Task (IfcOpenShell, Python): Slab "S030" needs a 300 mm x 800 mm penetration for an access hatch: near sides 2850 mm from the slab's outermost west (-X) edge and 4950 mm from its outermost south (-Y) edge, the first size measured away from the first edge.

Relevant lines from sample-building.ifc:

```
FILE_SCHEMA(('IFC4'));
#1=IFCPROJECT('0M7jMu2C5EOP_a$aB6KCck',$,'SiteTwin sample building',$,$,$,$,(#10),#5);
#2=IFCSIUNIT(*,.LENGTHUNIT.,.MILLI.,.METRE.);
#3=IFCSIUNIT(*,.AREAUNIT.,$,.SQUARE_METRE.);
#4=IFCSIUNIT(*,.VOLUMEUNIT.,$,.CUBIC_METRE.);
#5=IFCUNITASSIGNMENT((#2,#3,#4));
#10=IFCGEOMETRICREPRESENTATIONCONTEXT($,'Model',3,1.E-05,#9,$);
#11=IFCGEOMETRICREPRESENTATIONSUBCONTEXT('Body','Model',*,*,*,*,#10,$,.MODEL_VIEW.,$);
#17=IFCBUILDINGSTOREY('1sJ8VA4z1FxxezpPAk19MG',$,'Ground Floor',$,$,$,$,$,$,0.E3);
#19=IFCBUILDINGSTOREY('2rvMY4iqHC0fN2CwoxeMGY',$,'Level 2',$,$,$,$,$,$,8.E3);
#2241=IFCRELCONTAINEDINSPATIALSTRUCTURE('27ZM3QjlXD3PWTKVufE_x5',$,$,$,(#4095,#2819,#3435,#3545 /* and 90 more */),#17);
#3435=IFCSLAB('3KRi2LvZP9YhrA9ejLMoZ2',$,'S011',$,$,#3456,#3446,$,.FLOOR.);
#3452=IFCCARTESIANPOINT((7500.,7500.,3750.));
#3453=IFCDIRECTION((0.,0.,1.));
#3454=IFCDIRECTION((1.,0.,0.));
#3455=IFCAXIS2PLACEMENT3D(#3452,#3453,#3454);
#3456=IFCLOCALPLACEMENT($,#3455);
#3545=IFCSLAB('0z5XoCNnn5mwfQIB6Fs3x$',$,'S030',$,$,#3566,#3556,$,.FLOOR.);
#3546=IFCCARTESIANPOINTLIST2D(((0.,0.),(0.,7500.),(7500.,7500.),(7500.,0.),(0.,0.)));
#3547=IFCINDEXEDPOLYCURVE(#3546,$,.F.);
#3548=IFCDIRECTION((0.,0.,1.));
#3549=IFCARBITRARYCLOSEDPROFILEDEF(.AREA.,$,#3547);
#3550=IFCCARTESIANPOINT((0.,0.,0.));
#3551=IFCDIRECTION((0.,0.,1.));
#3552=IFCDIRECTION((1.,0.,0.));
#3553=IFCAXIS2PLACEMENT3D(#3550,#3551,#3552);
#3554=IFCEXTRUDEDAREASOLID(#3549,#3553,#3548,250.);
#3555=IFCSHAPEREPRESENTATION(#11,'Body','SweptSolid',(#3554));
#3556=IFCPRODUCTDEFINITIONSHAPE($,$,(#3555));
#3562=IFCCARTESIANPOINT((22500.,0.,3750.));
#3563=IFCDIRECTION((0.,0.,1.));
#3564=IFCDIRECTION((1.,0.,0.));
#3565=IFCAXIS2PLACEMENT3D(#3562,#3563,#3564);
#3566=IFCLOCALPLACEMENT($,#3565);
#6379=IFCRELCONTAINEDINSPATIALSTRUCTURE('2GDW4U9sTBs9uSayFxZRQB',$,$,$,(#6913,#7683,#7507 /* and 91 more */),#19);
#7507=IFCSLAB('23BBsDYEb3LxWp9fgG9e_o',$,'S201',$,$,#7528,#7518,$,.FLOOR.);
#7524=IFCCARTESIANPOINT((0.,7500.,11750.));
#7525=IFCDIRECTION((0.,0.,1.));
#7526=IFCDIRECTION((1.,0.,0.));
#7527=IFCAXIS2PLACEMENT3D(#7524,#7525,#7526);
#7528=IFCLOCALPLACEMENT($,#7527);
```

```python
import numpy as np
import ifcopenshell
import ifcopenshell.api.feature
import ifcopenshell.api.geometry
import ifcopenshell.api.root
import ifcopenshell.geom
import ifcopenshell.util.placement
import ifcopenshell.util.representation
import ifcopenshell.util.shape
import ifcopenshell.util.unit

model = ifcopenshell.open("sample-building.ifc")
unit_scale = ifcopenshell.util.unit.calculate_unit_scale(model)
settings = ifcopenshell.geom.settings()


def volume(element):
    """Net volume in cubic metres, openings subtracted."""
    shape = ifcopenshell.geom.create_shape(settings, element)
    return ifcopenshell.util.shape.get_volume(shape.geometry)


slab = model.by_guid("0z5XoCNnn5mwfQIB6Fs3x$")
before = volume(slab)

# Extent in the slab's own axes, in metres. The edges named are its -X and -Y sides.
slab_shape = ifcopenshell.geom.create_shape(settings, slab)
vertices = ifcopenshell.util.shape.get_vertices(slab_shape.geometry)
x_min, y_min, bottom = vertices.min(axis=0)
top = vertices[:, 2].max()

opening = ifcopenshell.api.root.create_entity(model, ifc_class="IfcOpeningElement", name="Access hatch opening", predefined_type="OPENING")
context = ifcopenshell.util.representation.get_context(model, "Model", "Body", "MODEL_VIEW")
width, depth = 0.3, 0.8
outline = [(0.0, 0.0), (width, 0.0), (width, depth), (0.0, depth), (0.0, 0.0)]
# Overshoot both faces by 50 mm so the cut is clean.
shape = ifcopenshell.api.geometry.add_slab_representation(
    model, context=context, depth=top - bottom + 0.1, polyline=outline
)
ifcopenshell.api.geometry.assign_representation(model, product=opening, representation=shape)

matrix = ifcopenshell.util.placement.get_local_placement(slab.ObjectPlacement)
matrix[:, 3] = matrix @ np.append(np.array([x_min + 2.85, y_min + 4.95, bottom - 0.05]) / unit_scale, 1.0)
ifcopenshell.api.geometry.edit_object_placement(model, product=opening, matrix=matrix, is_si=False)
ifcopenshell.api.feature.add_feature(model, feature=opening, element=slab)

after = volume(slab)

print(f"slab volume {before:.3f} -> {after:.3f} m3")

model.write("sample-building_updated.ifc")
```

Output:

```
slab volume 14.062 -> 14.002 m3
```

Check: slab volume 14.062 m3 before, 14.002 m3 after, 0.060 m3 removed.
